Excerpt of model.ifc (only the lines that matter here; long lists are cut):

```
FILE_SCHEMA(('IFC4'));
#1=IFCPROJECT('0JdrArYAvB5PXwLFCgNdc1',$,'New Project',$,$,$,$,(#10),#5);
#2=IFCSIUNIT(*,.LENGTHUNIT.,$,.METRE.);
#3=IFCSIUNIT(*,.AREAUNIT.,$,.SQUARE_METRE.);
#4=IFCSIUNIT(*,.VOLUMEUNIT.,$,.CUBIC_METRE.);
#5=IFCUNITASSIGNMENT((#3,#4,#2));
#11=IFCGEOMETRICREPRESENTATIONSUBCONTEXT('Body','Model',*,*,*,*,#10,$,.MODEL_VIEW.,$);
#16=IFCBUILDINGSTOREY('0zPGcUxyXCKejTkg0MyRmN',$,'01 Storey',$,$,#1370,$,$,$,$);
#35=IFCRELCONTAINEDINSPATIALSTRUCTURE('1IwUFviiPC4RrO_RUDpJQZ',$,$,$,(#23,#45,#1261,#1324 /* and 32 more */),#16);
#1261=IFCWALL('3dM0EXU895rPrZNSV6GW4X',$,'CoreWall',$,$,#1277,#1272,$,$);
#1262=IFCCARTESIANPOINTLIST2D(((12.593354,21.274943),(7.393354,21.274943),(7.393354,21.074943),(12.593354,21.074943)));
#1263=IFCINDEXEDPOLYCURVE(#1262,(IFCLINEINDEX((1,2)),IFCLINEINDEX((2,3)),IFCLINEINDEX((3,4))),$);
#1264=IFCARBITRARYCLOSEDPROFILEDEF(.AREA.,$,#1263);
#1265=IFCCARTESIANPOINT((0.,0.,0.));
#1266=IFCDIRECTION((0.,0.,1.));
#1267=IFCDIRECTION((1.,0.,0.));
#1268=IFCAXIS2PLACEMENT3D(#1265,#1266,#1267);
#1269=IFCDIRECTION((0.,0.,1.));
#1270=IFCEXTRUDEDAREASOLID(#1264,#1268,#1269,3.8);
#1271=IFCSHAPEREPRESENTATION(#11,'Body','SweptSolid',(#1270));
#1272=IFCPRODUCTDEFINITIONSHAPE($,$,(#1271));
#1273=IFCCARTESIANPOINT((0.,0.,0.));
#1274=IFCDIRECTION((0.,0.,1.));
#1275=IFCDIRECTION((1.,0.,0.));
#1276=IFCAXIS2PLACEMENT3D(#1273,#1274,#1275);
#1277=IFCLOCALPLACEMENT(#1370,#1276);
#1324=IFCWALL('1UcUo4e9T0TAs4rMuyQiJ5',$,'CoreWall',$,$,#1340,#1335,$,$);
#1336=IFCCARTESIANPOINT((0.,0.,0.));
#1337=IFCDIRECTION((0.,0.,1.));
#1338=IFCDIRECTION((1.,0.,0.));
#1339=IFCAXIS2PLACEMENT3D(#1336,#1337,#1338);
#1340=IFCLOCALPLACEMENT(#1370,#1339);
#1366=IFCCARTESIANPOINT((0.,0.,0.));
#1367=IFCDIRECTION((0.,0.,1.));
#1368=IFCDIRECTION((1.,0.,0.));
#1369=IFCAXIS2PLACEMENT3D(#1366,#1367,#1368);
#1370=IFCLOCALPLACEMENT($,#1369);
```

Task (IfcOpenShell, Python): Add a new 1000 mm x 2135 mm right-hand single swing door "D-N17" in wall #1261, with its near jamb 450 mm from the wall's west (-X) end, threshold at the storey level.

```python
import numpy as np
import ifcopenshell
import ifcopenshell.api.feature
import ifcopenshell.api.geometry
import ifcopenshell.api.root
import ifcopenshell.api.spatial
import ifcopenshell.geom
import ifcopenshell.util.element
import ifcopenshell.util.placement
import ifcopenshell.util.representation
import ifcopenshell.util.shape
import ifcopenshell.util.unit

model = ifcopenshell.open("model.ifc")
unit_scale = ifcopenshell.util.unit.calculate_unit_scale(model)
settings = ifcopenshell.geom.settings()


def volume(element):
    """Net volume in cubic metres, openings subtracted."""
    shape = ifcopenshell.geom.create_shape(settings, element)
    return ifcopenshell.util.shape.get_volume(shape.geometry)


wall = model.by_guid("3dM0EXU895rPrZNSV6GW4X")
storey = ifcopenshell.util.element.get_container(wall, ifc_class="IfcBuildingStorey")
context = ifcopenshell.util.representation.get_context(model, "Model", "Body", "MODEL_VIEW")
before = volume(wall)

width, height, from_end, sill = 1, 2.135, 0.45, 0.0  # metres

# The wall runs along its own X axis, and the end named is its -X end.
wall_shape = ifcopenshell.geom.create_shape(settings, wall)
x, y, z = ifcopenshell.util.shape.get_vertices(wall_shape.geometry).T
start = x.min() + from_end
face, thickness = float(y.min()), float(y.max() - y.min())
wall_matrix = ifcopenshell.util.placement.get_local_placement(wall.ObjectPlacement)
level = ifcopenshell.util.placement.get_local_placement(storey.ObjectPlacement)[2, 3]


def in_wall(x, y):
    """Placement at x, y metres in the wall's axes, at sill height."""
    matrix = wall_matrix.copy()
    matrix[:, 3] = wall_matrix @ np.array([x / unit_scale, y / unit_scale, 0.0, 1.0])
    matrix[2, 3] = level + sill / unit_scale
    return matrix


# Opening: a box that overshoots both wall faces by 50 mm.
opening = ifcopenshell.api.root.create_entity(model, ifc_class="IfcOpeningElement", predefined_type="OPENING")
box = ifcopenshell.api.geometry.add_wall_representation(
    model, context=context, length=width, height=height, thickness=thickness + 0.1
)
ifcopenshell.api.geometry.assign_representation(model, product=opening, representation=box)
ifcopenshell.api.geometry.edit_object_placement(model, product=opening, matrix=in_wall(start, face - 0.05), is_si=False)
ifcopenshell.api.feature.add_feature(model, feature=opening, element=wall)

door = ifcopenshell.api.root.create_entity(model, ifc_class="IfcDoor", name="D-N17", predefined_type="DOOR")
door.OverallWidth, door.OverallHeight = width / unit_scale, height / unit_scale
door.OperationType = "SINGLE_SWING_RIGHT"
body = ifcopenshell.api.geometry.add_door_representation(
    model,
    context=context,
    overall_width=door.OverallWidth,
    overall_height=door.OverallHeight,
    operation_type="SINGLE_SWING_RIGHT",
    lining_properties={"LiningDepth": thickness / unit_scale, "ThresholdDepth": thickness / unit_scale},
)
ifcopenshell.api.geometry.assign_representation(model, product=door, representation=body)
ifcopenshell.api.spatial.assign_container(model, products=[door], relating_structure=storey)
ifcopenshell.api.feature.add_filling(model, opening=opening, element=door)

# The lining spans the wall, so the door starts at the wall face.
ifcopenshell.api.geometry.edit_object_placement(model, product=door, matrix=in_wall(start, face), is_si=False)

after = volume(wall)

print(f"wall volume {before:.3f} -> {after:.3f} m3")

model.write("model-out.ifc")
```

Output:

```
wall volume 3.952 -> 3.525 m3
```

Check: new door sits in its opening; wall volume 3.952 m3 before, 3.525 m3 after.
